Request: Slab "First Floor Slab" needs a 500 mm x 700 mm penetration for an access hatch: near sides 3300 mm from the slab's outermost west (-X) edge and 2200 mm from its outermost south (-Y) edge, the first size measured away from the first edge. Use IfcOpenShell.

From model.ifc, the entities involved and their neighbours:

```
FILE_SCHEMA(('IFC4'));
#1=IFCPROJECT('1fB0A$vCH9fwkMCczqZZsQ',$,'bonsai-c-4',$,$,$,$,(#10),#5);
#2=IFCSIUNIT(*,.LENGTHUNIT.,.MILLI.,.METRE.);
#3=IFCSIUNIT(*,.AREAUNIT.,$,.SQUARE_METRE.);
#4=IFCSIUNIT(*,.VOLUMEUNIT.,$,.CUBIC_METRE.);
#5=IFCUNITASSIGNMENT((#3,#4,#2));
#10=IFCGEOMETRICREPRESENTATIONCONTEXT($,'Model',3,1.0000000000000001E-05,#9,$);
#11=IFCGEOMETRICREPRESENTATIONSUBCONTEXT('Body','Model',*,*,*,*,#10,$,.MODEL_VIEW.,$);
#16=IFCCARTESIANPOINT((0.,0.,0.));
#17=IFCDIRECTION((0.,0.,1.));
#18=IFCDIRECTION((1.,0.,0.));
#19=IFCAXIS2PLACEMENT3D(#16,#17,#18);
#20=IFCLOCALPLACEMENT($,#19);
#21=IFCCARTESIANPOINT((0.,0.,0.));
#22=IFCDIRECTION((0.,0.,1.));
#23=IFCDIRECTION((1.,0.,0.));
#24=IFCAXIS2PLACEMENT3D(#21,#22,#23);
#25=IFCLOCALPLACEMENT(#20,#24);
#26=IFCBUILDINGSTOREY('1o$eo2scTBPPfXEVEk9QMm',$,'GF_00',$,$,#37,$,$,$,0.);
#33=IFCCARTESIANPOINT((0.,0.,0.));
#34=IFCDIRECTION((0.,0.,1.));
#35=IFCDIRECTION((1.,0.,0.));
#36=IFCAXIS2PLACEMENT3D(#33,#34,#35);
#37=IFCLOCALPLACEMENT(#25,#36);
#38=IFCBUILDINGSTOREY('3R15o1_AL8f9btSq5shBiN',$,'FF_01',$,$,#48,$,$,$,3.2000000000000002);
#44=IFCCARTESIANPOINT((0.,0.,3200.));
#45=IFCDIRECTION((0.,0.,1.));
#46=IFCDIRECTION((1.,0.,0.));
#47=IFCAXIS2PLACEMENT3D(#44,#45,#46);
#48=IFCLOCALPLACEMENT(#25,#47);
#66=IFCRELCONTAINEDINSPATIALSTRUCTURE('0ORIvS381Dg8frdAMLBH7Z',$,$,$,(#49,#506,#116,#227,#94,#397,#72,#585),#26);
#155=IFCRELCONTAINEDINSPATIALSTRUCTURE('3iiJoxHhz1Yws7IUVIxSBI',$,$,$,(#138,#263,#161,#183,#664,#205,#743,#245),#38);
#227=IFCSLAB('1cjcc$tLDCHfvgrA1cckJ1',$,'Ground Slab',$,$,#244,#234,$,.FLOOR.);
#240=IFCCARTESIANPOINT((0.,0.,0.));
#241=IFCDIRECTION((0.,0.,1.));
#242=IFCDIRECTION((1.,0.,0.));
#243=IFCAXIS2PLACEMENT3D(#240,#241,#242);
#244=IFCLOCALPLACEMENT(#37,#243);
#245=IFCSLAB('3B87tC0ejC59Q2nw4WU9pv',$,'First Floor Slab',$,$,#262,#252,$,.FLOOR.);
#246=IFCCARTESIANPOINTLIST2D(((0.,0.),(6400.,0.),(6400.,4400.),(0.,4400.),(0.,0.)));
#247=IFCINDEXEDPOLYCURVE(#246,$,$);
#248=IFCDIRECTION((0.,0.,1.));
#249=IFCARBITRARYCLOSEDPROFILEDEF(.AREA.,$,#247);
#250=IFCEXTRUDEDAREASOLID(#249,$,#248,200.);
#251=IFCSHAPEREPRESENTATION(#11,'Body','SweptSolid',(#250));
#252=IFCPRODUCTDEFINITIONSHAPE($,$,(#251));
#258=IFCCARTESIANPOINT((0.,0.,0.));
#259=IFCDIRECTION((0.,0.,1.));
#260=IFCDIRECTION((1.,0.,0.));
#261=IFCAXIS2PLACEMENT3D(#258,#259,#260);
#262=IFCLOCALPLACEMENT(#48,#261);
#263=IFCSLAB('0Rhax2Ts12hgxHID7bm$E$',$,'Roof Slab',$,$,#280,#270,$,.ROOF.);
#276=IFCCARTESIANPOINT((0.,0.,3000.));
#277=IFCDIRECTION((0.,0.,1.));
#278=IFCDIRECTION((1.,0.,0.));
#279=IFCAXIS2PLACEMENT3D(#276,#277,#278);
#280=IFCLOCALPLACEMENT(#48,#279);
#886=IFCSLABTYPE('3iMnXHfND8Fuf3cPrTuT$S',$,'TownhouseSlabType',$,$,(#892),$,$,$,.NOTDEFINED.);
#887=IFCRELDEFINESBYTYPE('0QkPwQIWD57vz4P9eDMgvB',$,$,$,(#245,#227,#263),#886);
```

```python
import numpy as np
import ifcopenshell
import ifcopenshell.api.feature
import ifcopenshell.api.geometry
import ifcopenshell.api.root
import ifcopenshell.geom
import ifcopenshell.util.placement
import ifcopenshell.util.representation
import ifcopenshell.util.shape
import ifcopenshell.util.unit

model = ifcopenshell.open("model.ifc")
unit_scale = ifcopenshell.util.unit.calculate_unit_scale(model)
settings = ifcopenshell.geom.settings()


def volume(element):
    """Net volume in cubic metres, openings subtracted."""
    shape = ifcopenshell.geom.create_shape(settings, element)
    return ifcopenshell.util.shape.get_volume(shape.geometry)


slab = model.by_guid("3B87tC0ejC59Q2nw4WU9pv")
before = volume(slab)

# Extent in the slab's own axes, in metres. The edges named are its -X and -Y sides.
slab_shape = ifcopenshell.geom.create_shape(settings, slab)
vertices = ifcopenshell.util.shape.get_vertices(slab_shape.geometry)
x_min, y_min, bottom = vertices.min(axis=0)
top = vertices[:, 2].max()

opening = ifcopenshell.api.root.create_entity(model, ifc_class="IfcOpeningElement", name="Access hatch opening", predefined_type="OPENING")
context = ifcopenshell.util.representation.get_context(model, "Model", "Body", "MODEL_VIEW")
width, depth = 0.5, 0.7
outline = [(0.0, 0.0), (width, 0.0), (width, depth), (0.0, depth), (0.0, 0.0)]
# Overshoot both faces by 50 mm so the cut is clean.
shape = ifcopenshell.api.geometry.add_slab_representation(
    model, context=context, depth=top - bottom + 0.1, polyline=outline
)
ifcopenshell.api.geometry.assign_representation(model, product=opening, representation=shape)

matrix = ifcopenshell.util.placement.get_local_placement(slab.ObjectPlacement)
matrix[:, 3] = matrix @ np.append(np.array([x_min + 3.3, y_min + 2.2, bottom - 0.05]) / unit_scale, 1.0)
ifcopenshell.api.geometry.edit_object_placement(model, product=opening, matrix=matrix, is_si=False)
ifcopenshell.api.feature.add_feature(model, feature=opening, element=slab)

after = volume(slab)

print(f"slab volume {before:.3f} -> {after:.3f} m3")

model.write("model_rev.ifc")
```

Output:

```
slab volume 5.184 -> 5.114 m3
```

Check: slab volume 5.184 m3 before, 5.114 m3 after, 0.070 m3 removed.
